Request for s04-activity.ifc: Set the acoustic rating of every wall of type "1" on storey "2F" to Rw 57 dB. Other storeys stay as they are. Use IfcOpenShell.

First a look at what the model holds.

```python
import ifcopenshell
import ifcopenshell.util.element

model = ifcopenshell.open("s04-activity.ifc")
print(model.schema)
storey = next(s for s in model.by_type("IfcBuildingStorey") if s.Name == "2F")
walls = [e for e in ifcopenshell.util.element.get_decomposition(storey) if e.is_a("IfcWall")]
seen = {}
for e in walls:
    element_type = ifcopenshell.util.element.get_type(e)
    key = (element_type.Name if element_type != e and element_type else None, ifcopenshell.util.element.get_pset(e, "Pset_WallCommon", "AcousticRating"))
    seen[key] = seen.get(key, 0) + 1
for (name, value), count in sorted(seen.items(), key=str):
    print(count, "x", name, "|", value)
```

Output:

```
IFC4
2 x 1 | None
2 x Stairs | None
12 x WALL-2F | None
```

```python
import ifcopenshell
import ifcopenshell.api.pset
import ifcopenshell.util.element

model = ifcopenshell.open("s04-activity.ifc")

storey = next(s for s in model.by_type("IfcBuildingStorey") if s.Name == "2F")
walls = [e for e in ifcopenshell.util.element.get_decomposition(storey) if e.is_a("IfcWall")]

count = 0
for e in walls:
    element_type = ifcopenshell.util.element.get_type(e)
    if element_type in (None, e) or element_type.Name != "1":
        continue
    # add_pset returns the element's existing set when there is one.
    pset = ifcopenshell.api.pset.add_pset(model, product=e, name="Pset_WallCommon")
    ifcopenshell.api.pset.edit_pset(model, pset=pset, properties={"AcousticRating": "Rw 57 dB"})
    count += 1

print(count, "walls updated")

model.write("s04-activity_v2.ifc")
```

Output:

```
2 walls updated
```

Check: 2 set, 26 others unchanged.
